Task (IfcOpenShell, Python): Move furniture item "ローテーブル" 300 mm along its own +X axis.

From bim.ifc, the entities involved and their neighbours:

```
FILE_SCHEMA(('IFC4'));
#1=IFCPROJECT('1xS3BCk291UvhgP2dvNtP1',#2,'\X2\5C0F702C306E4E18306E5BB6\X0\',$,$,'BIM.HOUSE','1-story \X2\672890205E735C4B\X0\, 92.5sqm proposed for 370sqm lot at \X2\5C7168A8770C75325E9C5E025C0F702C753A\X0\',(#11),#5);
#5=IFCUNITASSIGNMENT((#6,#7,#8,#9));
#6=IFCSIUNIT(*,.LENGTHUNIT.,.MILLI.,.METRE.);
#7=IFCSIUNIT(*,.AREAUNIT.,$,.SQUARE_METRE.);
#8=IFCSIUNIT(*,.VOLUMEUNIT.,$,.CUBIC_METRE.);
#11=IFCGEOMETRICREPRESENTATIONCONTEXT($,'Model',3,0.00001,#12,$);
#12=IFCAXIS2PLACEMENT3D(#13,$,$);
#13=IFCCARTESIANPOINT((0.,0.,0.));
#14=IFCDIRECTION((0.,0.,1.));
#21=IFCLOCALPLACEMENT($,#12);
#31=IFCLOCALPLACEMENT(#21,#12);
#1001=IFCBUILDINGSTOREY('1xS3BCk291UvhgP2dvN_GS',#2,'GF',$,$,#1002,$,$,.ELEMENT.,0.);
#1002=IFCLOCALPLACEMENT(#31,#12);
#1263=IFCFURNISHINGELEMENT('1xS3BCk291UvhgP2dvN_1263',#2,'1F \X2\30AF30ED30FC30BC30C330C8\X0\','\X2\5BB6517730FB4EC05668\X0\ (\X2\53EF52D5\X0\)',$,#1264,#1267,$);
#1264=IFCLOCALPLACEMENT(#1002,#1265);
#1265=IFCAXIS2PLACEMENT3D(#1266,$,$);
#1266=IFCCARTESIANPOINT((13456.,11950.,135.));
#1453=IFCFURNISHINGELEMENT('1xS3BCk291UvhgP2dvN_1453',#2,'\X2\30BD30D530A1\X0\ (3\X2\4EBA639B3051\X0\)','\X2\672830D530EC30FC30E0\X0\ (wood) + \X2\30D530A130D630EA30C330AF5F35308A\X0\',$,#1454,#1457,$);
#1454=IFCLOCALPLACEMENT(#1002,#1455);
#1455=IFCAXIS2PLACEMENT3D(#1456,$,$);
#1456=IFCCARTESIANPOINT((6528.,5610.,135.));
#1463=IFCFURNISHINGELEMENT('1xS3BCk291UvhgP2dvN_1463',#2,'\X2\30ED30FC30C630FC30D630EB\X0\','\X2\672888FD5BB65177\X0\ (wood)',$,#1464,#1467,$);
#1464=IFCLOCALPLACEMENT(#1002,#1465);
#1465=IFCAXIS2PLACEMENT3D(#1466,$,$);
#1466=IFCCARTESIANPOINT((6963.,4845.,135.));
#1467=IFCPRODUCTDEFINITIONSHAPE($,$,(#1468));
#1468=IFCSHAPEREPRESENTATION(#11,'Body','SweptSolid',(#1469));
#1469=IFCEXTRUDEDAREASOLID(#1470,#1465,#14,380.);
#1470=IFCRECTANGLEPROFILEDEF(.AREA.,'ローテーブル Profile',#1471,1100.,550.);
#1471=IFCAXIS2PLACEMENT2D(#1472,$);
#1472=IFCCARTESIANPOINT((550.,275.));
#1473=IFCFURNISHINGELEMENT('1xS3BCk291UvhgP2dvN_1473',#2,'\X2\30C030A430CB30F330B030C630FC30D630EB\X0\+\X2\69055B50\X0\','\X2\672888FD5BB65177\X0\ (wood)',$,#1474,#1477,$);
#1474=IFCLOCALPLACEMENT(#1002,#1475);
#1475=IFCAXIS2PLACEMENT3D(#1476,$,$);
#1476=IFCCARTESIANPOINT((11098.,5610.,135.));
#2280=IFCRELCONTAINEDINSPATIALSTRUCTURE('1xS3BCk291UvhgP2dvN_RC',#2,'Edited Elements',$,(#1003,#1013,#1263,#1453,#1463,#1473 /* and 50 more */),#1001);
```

```python
import ifcopenshell
import ifcopenshell.api.geometry
import ifcopenshell.util.placement
import ifcopenshell.util.unit

model = ifcopenshell.open("bim.ifc")
unit_scale = ifcopenshell.util.unit.calculate_unit_scale(model)

item = model.by_guid("1xS3BCk291UvhgP2dvN_1463")
matrix = ifcopenshell.util.placement.get_local_placement(item.ObjectPlacement)
matrix[:3, 3] += matrix[:3, 0] * 0.3 / unit_scale
ifcopenshell.api.geometry.edit_object_placement(model, product=item, matrix=matrix, is_si=False)

print(ifcopenshell.util.placement.get_local_placement(item.ObjectPlacement).round(3) + 0.0)

model.write("bim_updated.ifc")
```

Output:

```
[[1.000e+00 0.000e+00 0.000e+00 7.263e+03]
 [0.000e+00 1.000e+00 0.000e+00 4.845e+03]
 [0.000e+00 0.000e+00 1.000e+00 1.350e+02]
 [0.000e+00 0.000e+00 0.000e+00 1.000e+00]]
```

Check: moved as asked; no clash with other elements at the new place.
